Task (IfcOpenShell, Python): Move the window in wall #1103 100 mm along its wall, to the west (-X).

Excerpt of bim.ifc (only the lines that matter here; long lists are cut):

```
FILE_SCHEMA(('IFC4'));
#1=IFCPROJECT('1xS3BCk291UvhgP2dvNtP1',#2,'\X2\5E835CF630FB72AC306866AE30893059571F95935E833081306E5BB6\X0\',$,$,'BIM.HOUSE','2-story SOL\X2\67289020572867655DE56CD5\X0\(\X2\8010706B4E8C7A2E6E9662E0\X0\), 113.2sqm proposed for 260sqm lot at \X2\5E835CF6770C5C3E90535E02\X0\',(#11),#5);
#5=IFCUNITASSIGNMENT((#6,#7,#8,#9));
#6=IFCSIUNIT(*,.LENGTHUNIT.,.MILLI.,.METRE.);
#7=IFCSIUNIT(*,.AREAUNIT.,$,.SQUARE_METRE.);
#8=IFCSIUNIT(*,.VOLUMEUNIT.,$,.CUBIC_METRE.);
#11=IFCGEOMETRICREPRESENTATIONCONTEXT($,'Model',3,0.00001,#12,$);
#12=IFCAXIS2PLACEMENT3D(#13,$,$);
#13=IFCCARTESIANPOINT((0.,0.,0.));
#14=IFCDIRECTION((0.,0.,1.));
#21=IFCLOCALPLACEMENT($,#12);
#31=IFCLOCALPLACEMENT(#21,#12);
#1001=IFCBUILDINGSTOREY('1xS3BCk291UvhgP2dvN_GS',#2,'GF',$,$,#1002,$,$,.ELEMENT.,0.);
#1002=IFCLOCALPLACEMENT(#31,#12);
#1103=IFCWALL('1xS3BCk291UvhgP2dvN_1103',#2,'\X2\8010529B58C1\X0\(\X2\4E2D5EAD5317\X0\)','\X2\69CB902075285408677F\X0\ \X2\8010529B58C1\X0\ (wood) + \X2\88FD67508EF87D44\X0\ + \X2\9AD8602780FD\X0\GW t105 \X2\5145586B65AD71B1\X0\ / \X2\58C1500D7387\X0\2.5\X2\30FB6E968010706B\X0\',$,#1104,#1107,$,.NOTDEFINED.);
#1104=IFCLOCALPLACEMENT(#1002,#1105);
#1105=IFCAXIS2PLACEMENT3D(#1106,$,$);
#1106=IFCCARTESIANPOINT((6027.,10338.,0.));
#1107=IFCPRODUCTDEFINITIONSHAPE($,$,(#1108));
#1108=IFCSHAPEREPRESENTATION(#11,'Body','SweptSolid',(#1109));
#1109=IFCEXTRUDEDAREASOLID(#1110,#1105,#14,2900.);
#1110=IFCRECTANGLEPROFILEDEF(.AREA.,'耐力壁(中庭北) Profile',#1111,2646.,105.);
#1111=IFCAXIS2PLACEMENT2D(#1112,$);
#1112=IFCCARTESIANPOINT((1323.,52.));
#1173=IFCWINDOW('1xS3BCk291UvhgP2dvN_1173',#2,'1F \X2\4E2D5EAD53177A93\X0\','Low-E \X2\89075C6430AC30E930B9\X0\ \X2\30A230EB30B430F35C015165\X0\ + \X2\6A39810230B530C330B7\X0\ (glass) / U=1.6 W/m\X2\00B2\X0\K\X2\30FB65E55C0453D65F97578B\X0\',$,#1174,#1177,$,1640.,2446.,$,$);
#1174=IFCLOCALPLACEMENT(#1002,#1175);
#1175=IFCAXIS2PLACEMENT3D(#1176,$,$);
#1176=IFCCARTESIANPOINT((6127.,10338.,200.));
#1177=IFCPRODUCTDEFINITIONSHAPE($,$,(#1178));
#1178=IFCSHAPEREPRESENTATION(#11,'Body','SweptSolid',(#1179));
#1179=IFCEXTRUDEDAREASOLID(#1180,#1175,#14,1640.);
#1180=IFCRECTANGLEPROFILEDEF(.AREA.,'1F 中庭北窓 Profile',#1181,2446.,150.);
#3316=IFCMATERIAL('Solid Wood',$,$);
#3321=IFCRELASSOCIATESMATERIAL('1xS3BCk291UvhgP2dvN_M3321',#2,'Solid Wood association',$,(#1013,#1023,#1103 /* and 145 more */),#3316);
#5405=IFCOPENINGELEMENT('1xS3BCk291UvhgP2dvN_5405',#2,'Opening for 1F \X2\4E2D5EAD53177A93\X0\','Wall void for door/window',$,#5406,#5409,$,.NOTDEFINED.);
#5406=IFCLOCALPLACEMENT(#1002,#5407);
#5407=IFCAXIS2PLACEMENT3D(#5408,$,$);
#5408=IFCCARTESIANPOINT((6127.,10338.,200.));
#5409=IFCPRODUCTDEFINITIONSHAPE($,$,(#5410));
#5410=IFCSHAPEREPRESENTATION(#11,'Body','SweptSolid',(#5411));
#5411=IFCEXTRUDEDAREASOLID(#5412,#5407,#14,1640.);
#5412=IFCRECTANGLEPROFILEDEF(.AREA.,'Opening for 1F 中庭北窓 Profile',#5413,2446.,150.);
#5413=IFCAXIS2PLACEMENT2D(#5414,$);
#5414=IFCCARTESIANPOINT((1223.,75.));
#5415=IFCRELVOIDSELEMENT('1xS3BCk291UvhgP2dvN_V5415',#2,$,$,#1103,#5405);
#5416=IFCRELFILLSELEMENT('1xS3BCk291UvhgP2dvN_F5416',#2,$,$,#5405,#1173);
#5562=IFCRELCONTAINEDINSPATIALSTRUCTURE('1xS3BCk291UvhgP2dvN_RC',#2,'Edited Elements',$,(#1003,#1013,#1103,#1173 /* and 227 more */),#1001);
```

```python
import ifcopenshell
import ifcopenshell.api.geometry
import ifcopenshell.util.placement
import ifcopenshell.util.unit

model = ifcopenshell.open("bim.ifc")
unit_scale = ifcopenshell.util.unit.calculate_unit_scale(model)

window = model.by_guid("1xS3BCk291UvhgP2dvN_1173")
opening = window.FillsVoids[0].RelatingOpeningElement
wall = opening.VoidsElements[0].RelatingBuildingElement

wall_matrix = ifcopenshell.util.placement.get_local_placement(wall.ObjectPlacement)
shift = wall_matrix[:3, 0] * -0.1 / unit_scale
before = ifcopenshell.util.placement.get_local_placement(window.ObjectPlacement)[:3, 3].copy()

# The window is not placed relative to its opening, so move both.
for product in (opening, window):
    matrix = ifcopenshell.util.placement.get_local_placement(product.ObjectPlacement)
    matrix[:3, 3] += shift
    ifcopenshell.api.geometry.edit_object_placement(model, product=product, matrix=matrix, is_si=False)

after = ifcopenshell.util.placement.get_local_placement(window.ObjectPlacement)[:3, 3]
print("window moved by", (after - before).round(3) + 0.0)

model.write("bim_updated.ifc")
```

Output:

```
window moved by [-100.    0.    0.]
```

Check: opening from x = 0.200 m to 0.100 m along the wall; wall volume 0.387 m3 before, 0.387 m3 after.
